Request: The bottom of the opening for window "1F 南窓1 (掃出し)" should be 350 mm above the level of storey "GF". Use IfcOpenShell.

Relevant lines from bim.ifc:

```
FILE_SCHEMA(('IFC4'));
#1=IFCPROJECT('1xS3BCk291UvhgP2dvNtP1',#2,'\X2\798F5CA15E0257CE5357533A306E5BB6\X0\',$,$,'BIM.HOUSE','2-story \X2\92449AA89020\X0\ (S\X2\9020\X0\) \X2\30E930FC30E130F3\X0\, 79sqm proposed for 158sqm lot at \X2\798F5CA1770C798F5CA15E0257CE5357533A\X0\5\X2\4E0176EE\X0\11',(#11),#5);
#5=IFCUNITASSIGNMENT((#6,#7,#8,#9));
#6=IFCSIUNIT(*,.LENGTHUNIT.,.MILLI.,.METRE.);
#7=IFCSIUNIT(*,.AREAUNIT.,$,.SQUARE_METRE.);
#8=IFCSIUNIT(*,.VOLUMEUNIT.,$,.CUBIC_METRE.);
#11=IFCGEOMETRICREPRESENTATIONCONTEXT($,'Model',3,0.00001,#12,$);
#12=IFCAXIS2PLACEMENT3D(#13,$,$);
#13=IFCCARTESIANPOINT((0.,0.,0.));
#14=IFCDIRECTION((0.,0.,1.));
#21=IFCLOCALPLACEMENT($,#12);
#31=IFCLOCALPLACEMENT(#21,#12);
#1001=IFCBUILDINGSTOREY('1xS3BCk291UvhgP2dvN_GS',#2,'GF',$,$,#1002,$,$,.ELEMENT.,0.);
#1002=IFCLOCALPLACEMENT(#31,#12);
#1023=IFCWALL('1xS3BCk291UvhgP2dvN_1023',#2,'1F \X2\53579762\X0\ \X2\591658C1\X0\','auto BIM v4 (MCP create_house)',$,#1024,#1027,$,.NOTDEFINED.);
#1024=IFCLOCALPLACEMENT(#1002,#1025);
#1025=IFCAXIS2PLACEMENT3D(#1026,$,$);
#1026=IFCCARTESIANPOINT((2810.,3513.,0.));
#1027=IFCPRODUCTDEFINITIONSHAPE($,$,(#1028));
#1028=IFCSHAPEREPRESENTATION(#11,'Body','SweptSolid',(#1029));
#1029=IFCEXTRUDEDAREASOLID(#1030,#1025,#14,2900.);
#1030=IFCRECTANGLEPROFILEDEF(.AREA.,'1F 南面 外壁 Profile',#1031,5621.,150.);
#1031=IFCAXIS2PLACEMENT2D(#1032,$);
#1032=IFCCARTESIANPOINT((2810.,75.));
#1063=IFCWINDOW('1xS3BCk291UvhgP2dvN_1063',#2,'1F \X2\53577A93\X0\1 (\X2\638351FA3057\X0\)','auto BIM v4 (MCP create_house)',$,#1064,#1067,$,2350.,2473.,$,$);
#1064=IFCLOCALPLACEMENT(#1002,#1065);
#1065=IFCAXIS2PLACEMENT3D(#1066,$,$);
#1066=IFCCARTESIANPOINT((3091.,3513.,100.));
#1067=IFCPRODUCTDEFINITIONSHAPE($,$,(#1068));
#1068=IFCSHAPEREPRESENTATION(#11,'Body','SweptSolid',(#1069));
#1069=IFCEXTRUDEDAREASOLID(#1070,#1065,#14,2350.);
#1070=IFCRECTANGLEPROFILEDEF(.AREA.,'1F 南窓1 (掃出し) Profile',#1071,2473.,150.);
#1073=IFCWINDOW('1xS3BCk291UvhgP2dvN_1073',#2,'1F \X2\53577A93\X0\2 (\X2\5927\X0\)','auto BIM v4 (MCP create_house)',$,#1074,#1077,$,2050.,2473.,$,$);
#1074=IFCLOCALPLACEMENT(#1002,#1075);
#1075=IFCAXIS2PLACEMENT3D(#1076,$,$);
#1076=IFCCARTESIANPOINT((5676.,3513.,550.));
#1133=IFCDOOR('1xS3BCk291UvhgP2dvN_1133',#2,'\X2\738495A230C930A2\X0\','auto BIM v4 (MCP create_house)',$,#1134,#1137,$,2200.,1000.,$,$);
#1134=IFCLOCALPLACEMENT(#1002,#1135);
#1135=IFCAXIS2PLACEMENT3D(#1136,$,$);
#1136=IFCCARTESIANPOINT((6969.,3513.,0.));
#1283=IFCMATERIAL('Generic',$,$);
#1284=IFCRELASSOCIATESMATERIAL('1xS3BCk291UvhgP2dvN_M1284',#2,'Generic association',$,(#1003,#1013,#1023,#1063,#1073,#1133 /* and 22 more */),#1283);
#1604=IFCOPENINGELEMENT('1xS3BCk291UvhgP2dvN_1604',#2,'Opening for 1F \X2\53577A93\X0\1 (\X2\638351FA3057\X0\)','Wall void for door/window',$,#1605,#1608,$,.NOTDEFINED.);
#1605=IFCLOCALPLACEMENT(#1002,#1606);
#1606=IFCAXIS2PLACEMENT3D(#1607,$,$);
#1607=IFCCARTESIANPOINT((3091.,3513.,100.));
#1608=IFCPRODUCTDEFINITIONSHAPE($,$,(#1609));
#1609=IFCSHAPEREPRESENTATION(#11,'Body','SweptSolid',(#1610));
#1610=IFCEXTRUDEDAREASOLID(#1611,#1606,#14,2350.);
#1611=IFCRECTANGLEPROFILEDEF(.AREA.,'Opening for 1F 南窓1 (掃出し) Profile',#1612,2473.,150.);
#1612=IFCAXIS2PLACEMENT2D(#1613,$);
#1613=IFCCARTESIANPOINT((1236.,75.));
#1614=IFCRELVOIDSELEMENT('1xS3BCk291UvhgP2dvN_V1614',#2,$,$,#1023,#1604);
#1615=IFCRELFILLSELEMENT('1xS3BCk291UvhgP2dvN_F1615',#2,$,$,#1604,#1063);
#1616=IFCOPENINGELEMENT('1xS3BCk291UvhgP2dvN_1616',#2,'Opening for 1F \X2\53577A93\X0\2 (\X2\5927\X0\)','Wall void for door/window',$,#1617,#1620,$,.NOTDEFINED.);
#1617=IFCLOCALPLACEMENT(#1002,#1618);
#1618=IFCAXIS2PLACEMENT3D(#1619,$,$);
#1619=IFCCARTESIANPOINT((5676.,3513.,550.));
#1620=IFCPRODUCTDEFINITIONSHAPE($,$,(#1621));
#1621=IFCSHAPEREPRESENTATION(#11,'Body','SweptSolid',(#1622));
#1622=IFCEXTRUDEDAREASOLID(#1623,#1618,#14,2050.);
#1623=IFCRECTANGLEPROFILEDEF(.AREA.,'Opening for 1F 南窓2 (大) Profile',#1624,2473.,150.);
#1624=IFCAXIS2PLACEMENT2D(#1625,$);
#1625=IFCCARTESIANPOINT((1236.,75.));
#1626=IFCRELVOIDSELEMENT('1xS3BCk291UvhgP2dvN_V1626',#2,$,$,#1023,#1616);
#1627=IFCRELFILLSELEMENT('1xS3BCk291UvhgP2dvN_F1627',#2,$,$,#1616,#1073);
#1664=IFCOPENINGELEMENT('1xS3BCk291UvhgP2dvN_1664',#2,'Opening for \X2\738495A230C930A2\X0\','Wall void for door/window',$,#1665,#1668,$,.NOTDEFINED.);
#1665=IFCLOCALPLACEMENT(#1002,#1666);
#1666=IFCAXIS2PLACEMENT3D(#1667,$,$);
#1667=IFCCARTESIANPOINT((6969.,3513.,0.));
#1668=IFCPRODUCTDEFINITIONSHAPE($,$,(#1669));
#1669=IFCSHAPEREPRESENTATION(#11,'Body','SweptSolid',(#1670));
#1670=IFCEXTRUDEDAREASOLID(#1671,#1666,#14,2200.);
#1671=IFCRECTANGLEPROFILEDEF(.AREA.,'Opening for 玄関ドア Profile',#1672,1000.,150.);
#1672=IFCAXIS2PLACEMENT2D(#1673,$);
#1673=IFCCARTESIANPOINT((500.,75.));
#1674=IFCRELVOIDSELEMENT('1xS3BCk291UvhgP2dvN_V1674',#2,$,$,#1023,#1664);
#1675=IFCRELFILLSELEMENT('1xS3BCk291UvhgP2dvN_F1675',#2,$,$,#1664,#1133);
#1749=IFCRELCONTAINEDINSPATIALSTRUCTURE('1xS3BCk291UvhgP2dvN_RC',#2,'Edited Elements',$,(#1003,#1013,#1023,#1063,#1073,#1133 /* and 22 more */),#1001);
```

```python
import numpy as np
import ifcopenshell
import ifcopenshell.api.geometry
import ifcopenshell.geom
import ifcopenshell.util.element
import ifcopenshell.util.placement
import ifcopenshell.util.shape
import ifcopenshell.util.unit

model = ifcopenshell.open("bim.ifc")
unit_scale = ifcopenshell.util.unit.calculate_unit_scale(model)

window = model.by_guid("1xS3BCk291UvhgP2dvN_1063")
opening = window.FillsVoids[0].RelatingOpeningElement
storey = ifcopenshell.util.element.get_container(window, ifc_class="IfcBuildingStorey")
level = ifcopenshell.util.placement.get_local_placement(storey.ObjectPlacement)[2, 3]

# The opening's origin need not be at the sill, so measure its lowest point.
shape = ifcopenshell.geom.create_shape(ifcopenshell.geom.settings(), opening)
bottom = ifcopenshell.util.shape.get_shape_bottom_elevation(shape, shape.geometry) / unit_scale
dz = level + 350.0 - bottom

shift = np.array([0.0, 0.0, dz])
# The window is not placed relative to its opening, so move both.
for product in (opening, window):
    matrix = ifcopenshell.util.placement.get_local_placement(product.ObjectPlacement)
    matrix[:3, 3] += shift
    ifcopenshell.api.geometry.edit_object_placement(model, product=product, matrix=matrix, is_si=False)

print(f"moved by {dz * unit_scale:+.3f} m")

model.write("bim_edited.ifc")
```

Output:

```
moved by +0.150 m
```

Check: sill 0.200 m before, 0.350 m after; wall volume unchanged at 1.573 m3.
